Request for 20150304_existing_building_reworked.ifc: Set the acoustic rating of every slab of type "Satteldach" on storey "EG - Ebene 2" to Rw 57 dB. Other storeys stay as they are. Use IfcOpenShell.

First a look at what the model holds.

```python
import ifcopenshell
import ifcopenshell.util.element

model = ifcopenshell.open("20150304_existing_building_reworked.ifc")
print(model.schema)
storey = next(s for s in model.by_type("IfcBuildingStorey") if s.Name == "EG - Ebene 2")
slabs = [e for e in ifcopenshell.util.element.get_decomposition(storey) if e.is_a("IfcSlab")]
seen = {}
for e in slabs:
    element_type = ifcopenshell.util.element.get_type(e)
    key = (element_type.Name if element_type != e and element_type else None, ifcopenshell.util.element.get_pset(e, "Pset_SlabCommon", "AcousticRating"))
    seen[key] = seen.get(key, 0) + 1
for (name, value), count in sorted(seen.items(), key=str):
    print(count, "x", name, "|", value)
```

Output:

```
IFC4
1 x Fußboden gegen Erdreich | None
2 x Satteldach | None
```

```python
import ifcopenshell
import ifcopenshell.api.pset
import ifcopenshell.util.element

model = ifcopenshell.open("20150304_existing_building_reworked.ifc")

storey = next(s for s in model.by_type("IfcBuildingStorey") if s.Name == "EG - Ebene 2")
slabs = [e for e in ifcopenshell.util.element.get_decomposition(storey) if e.is_a("IfcSlab")]

count = 0
for e in slabs:
    element_type = ifcopenshell.util.element.get_type(e)
    if element_type in (None, e) or element_type.Name != "Satteldach":
        continue
    # add_pset returns the element's existing set when there is one.
    pset = ifcopenshell.api.pset.add_pset(model, product=e, name="Pset_SlabCommon")
    ifcopenshell.api.pset.edit_pset(model, pset=pset, properties={"AcousticRating": "Rw 57 dB"})
    count += 1

print(count, "slabs updated")

model.write("20150304_existing_building_reworked_rev.ifc")
```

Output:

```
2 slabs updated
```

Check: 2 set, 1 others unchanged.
